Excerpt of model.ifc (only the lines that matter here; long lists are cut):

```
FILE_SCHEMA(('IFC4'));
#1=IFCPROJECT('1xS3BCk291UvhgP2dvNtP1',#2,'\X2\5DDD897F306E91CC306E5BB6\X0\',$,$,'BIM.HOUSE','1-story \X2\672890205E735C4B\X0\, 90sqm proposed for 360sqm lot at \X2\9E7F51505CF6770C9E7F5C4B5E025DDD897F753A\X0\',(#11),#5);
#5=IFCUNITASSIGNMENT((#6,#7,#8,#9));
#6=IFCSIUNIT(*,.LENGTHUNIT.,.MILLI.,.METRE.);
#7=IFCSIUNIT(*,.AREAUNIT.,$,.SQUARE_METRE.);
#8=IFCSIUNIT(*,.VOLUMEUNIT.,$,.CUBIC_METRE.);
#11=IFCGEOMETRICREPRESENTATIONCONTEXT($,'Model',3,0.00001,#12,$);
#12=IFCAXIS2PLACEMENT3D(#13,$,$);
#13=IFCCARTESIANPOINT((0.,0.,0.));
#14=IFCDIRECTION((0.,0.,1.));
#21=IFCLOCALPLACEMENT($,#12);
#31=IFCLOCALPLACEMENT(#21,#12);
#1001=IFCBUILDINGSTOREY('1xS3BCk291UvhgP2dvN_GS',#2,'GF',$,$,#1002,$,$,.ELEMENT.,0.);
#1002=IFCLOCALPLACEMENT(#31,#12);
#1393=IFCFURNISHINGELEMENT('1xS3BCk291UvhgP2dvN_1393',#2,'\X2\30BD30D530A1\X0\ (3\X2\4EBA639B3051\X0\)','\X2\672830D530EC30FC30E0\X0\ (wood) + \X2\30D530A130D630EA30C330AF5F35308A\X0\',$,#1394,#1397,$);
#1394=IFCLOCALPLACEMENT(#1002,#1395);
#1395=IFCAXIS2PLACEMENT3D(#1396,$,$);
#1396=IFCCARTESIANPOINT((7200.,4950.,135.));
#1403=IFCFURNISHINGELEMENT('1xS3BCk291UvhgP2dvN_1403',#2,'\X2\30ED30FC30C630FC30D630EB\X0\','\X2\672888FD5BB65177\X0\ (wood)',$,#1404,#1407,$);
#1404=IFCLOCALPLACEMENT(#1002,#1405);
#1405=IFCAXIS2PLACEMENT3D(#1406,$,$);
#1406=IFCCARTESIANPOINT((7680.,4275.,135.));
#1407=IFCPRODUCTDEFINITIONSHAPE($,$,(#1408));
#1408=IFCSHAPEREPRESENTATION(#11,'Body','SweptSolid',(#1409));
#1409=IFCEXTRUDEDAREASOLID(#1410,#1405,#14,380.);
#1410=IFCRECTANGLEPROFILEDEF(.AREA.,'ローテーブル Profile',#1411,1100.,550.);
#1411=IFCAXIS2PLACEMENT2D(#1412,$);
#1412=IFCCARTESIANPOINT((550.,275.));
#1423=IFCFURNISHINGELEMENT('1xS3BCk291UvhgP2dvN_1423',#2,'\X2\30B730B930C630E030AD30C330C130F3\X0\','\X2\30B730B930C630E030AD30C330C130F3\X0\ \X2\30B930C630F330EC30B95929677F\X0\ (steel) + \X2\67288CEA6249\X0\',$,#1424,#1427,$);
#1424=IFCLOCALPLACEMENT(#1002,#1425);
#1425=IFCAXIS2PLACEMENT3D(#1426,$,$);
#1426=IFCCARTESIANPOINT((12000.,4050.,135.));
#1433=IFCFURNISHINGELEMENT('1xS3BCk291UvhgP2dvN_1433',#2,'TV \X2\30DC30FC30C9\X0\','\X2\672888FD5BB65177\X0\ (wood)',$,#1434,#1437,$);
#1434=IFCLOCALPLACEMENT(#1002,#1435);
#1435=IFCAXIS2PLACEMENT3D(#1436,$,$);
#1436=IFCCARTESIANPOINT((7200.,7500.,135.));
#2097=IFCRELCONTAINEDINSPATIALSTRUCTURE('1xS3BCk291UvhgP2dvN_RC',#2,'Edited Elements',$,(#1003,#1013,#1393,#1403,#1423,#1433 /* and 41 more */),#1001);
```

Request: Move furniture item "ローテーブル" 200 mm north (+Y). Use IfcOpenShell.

```python
import ifcopenshell
import ifcopenshell.api.geometry
import ifcopenshell.util.placement
import ifcopenshell.util.unit

model = ifcopenshell.open("model.ifc")
unit_scale = ifcopenshell.util.unit.calculate_unit_scale(model)

item = model.by_guid("1xS3BCk291UvhgP2dvN_1403")
matrix = ifcopenshell.util.placement.get_local_placement(item.ObjectPlacement)
matrix[1, 3] += 0.2 / unit_scale
ifcopenshell.api.geometry.edit_object_placement(model, product=item, matrix=matrix, is_si=False)

print(ifcopenshell.util.placement.get_local_placement(item.ObjectPlacement).round(3) + 0.0)

model.write("model_v2.ifc")
```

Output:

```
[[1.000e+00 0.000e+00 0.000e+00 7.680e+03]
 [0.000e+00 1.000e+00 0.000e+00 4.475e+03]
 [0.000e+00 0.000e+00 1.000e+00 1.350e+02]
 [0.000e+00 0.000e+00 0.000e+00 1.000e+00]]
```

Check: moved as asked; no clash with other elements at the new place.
